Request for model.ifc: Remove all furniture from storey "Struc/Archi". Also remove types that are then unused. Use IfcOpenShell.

First a look at what the model holds.

```python
import ifcopenshell
import ifcopenshell.util.element

model = ifcopenshell.open("model.ifc")
print(model.schema)
storey = next(s for s in model.by_type("IfcBuildingStorey") if s.Name == "Struc/Archi")
furniture = [e for e in ifcopenshell.util.element.get_decomposition(storey) if e.is_a("IfcFurnishingElement")]
seen = {}
for e in furniture:
    element_type = ifcopenshell.util.element.get_type(e)
    name = element_type.Name if element_type not in (None, e) else None
    seen[name] = seen.get(name, 0) + 1
for name, count in sorted(seen.items(), key=str):
    print(count, "x", name)
```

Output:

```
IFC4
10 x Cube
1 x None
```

```python
import ifcopenshell
import ifcopenshell.api.root
import ifcopenshell.util.element

model = ifcopenshell.open("model.ifc")

storey = next(s for s in model.by_type("IfcBuildingStorey") if s.Name == "Struc/Archi")
furniture = [e for e in ifcopenshell.util.element.get_decomposition(storey) if e.is_a("IfcFurnishingElement")]
types = {ifcopenshell.util.element.get_type(e) for e in furniture} - {None, *furniture}

for e in furniture:
    ifcopenshell.api.root.remove_product(model, product=e)
print(len(furniture), "removed")

unused = [t for t in types if not ifcopenshell.util.element.get_types(t)]
for t in unused:
    ifcopenshell.api.root.remove_product(model, product=t)
print(len(unused), "unused types removed")

model.write("model_v2.ifc")
```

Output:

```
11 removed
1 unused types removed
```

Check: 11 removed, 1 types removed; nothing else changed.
